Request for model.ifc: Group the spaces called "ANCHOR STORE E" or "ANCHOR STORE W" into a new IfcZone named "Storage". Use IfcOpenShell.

First a look at what the model holds.

```python
import ifcopenshell

model = ifcopenshell.open("model.ifc")
print(model.schema)
seen = {}
for space in model.by_type("IfcSpace"):
    seen[space.LongName] = seen.get(space.LongName, 0) + 1
for name, count in sorted(seen.items(), key=str):
    print(count, "x", name)
print("zones:", [z.Name for z in model.by_type("IfcZone")][:20])
```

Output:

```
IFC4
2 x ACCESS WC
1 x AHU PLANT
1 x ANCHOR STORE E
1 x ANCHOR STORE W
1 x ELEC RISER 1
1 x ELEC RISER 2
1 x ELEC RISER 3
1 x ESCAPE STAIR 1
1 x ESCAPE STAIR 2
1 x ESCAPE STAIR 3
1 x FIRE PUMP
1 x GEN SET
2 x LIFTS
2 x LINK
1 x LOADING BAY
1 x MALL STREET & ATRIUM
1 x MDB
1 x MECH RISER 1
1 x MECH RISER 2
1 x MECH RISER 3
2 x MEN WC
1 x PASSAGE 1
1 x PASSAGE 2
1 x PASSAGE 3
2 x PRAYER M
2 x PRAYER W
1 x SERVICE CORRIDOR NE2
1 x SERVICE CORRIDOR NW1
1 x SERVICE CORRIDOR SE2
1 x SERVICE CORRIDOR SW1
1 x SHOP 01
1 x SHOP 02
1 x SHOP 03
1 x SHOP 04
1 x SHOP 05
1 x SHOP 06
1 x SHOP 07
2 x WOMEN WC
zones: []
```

```python
import ifcopenshell
import ifcopenshell.api.group
import ifcopenshell.api.root

model = ifcopenshell.open("model.ifc")

names = {"ANCHOR STORE E", "ANCHOR STORE W"}
spaces = [s for s in model.by_type("IfcSpace") if s.LongName in names]

zone = ifcopenshell.api.root.create_entity(model, ifc_class="IfcZone", name="Storage")
ifcopenshell.api.group.assign_group(model, products=spaces, group=zone)
print(len(spaces), "spaces in", zone.Name)

model.write("model_v2.ifc")
```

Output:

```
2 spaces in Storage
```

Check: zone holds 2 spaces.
